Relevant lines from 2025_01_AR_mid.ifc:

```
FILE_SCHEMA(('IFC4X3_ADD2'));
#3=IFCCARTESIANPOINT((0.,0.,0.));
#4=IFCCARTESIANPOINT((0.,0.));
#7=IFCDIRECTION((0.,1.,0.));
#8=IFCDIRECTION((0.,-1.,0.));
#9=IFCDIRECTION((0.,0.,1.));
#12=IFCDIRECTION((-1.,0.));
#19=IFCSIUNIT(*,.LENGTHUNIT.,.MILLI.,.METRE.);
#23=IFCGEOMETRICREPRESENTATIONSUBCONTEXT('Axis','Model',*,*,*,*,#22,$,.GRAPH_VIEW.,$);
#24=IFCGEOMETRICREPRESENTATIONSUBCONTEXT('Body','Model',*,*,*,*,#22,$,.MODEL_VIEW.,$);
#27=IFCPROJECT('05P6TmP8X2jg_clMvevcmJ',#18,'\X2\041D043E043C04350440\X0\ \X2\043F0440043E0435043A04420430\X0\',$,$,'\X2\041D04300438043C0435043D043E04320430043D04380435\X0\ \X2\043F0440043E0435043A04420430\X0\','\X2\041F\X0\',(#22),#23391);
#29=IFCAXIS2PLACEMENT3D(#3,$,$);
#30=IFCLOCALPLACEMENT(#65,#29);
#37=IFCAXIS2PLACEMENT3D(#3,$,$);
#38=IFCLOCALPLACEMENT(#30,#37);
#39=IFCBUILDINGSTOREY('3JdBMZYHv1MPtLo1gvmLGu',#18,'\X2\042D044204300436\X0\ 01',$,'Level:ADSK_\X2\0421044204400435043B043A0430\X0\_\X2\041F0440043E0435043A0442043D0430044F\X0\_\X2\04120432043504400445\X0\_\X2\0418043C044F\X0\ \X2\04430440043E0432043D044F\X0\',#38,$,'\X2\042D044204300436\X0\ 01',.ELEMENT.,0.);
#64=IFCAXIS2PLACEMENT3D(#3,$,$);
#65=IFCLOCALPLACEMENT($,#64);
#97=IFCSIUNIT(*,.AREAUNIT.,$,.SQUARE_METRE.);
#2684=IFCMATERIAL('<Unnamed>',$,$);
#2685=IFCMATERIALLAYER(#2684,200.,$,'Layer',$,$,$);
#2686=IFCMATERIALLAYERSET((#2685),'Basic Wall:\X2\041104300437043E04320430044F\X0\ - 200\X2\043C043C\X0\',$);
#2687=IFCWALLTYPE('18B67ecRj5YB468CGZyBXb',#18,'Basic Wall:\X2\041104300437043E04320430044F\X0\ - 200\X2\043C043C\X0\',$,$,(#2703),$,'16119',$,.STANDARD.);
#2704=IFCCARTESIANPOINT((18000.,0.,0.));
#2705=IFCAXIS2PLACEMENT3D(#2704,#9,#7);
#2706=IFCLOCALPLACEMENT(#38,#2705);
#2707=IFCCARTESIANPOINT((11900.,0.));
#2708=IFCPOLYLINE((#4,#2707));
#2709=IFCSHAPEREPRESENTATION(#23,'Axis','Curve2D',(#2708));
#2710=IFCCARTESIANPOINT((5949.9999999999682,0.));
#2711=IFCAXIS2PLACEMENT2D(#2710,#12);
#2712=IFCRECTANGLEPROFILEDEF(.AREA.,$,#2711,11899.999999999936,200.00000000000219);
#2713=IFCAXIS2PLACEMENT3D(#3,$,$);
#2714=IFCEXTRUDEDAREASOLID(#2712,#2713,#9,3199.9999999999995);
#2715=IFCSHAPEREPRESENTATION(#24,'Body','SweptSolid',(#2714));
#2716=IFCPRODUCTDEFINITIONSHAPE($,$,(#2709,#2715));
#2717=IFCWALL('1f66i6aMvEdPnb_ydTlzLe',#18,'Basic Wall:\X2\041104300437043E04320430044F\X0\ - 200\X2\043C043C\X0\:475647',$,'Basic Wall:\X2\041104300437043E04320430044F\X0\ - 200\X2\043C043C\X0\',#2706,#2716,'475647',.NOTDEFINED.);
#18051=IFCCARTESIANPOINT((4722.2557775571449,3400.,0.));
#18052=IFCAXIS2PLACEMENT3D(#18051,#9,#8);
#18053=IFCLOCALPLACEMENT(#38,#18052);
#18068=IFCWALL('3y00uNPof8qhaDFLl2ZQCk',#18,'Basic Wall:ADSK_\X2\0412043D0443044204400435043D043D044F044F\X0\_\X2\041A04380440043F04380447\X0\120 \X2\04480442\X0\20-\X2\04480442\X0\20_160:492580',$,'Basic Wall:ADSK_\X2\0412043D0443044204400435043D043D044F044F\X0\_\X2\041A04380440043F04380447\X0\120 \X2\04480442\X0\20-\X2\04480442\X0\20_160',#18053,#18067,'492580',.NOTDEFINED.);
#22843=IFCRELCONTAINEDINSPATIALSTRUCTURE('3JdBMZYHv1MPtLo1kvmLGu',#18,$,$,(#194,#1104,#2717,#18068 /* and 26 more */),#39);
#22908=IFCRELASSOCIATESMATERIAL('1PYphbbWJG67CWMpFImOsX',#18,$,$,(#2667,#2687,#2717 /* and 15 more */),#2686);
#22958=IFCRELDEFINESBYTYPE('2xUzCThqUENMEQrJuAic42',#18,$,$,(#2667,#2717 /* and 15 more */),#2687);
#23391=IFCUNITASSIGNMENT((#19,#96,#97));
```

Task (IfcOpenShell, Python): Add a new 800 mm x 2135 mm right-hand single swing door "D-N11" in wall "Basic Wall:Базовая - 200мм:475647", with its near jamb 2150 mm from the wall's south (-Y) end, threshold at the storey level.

```python
import numpy as np
import ifcopenshell
import ifcopenshell.api.feature
import ifcopenshell.api.geometry
import ifcopenshell.api.root
import ifcopenshell.api.spatial
import ifcopenshell.geom
import ifcopenshell.util.element
import ifcopenshell.util.placement
import ifcopenshell.util.representation
import ifcopenshell.util.shape
import ifcopenshell.util.unit

model = ifcopenshell.open("2025_01_AR_mid.ifc")
unit_scale = ifcopenshell.util.unit.calculate_unit_scale(model)
settings = ifcopenshell.geom.settings()


def volume(element):
    """Net volume in cubic metres, openings subtracted."""
    shape = ifcopenshell.geom.create_shape(settings, element)
    return ifcopenshell.util.shape.get_volume(shape.geometry)


wall = model.by_guid("1f66i6aMvEdPnb_ydTlzLe")
storey = ifcopenshell.util.element.get_container(wall, ifc_class="IfcBuildingStorey")
context = ifcopenshell.util.representation.get_context(model, "Model", "Body", "MODEL_VIEW")
before = volume(wall)

width, height, from_end, sill = 0.8, 2.135, 2.15, 0.0  # metres

# The wall runs along its own X axis, and the end named is its -X end.
wall_shape = ifcopenshell.geom.create_shape(settings, wall)
x, y, z = ifcopenshell.util.shape.get_vertices(wall_shape.geometry).T
start = x.min() + from_end
face, thickness = float(y.min()), float(y.max() - y.min())
wall_matrix = ifcopenshell.util.placement.get_local_placement(wall.ObjectPlacement)
level = ifcopenshell.util.placement.get_local_placement(storey.ObjectPlacement)[2, 3]


def in_wall(x, y):
    """Placement at x, y metres in the wall's axes, at sill height."""
    matrix = wall_matrix.copy()
    matrix[:, 3] = wall_matrix @ np.array([x / unit_scale, y / unit_scale, 0.0, 1.0])
    matrix[2, 3] = level + sill / unit_scale
    return matrix


# Opening: a box that overshoots both wall faces by 50 mm.
opening = ifcopenshell.api.root.create_entity(model, ifc_class="IfcOpeningElement", predefined_type="OPENING")
box = ifcopenshell.api.geometry.add_wall_representation(
    model, context=context, length=width, height=height, thickness=thickness + 0.1
)
ifcopenshell.api.geometry.assign_representation(model, product=opening, representation=box)
ifcopenshell.api.geometry.edit_object_placement(model, product=opening, matrix=in_wall(start, face - 0.05), is_si=False)
ifcopenshell.api.feature.add_feature(model, feature=opening, element=wall)

door = ifcopenshell.api.root.create_entity(model, ifc_class="IfcDoor", name="D-N11", predefined_type="DOOR")
door.OverallWidth, door.OverallHeight = width / unit_scale, height / unit_scale
door.OperationType = "SINGLE_SWING_RIGHT"
body = ifcopenshell.api.geometry.add_door_representation(
    model,
    context=context,
    overall_width=door.OverallWidth,
    overall_height=door.OverallHeight,
    operation_type="SINGLE_SWING_RIGHT",
    lining_properties={"LiningDepth": thickness / unit_scale, "ThresholdDepth": thickness / unit_scale},
)
ifcopenshell.api.geometry.assign_representation(model, product=door, representation=body)
ifcopenshell.api.spatial.assign_container(model, products=[door], relating_structure=storey)
ifcopenshell.api.feature.add_filling(model, opening=opening, element=door)

# The lining spans the wall, so the door starts at the wall face.
ifcopenshell.api.geometry.edit_object_placement(model, product=door, matrix=in_wall(start, face), is_si=False)

after = volume(wall)

print(f"wall volume {before:.3f} -> {after:.3f} m3")

model.write("2025_01_AR_mid-out.ifc")
```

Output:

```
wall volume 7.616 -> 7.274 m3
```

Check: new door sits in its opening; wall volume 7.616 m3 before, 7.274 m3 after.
